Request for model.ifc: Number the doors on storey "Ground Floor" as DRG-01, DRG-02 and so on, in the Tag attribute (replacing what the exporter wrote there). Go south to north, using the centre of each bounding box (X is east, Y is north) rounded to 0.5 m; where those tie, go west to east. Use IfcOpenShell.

First a look at what the model holds.

```python
import ifcopenshell
import ifcopenshell.util.element
import ifcopenshell.util.placement

model = ifcopenshell.open("model.ifc")
print(model.schema)
storey = next(s for s in model.by_type("IfcBuildingStorey") if s.Name == "Ground Floor")
doors = [e for e in ifcopenshell.util.element.get_decomposition(storey) if e.is_a("IfcDoor")]
for e in sorted(doors, key=lambda e: e.id()):
    origin = ifcopenshell.util.placement.get_local_placement(e.ObjectPlacement)[:3, 3]
    print(e.id(), e.Tag, e.Name, origin.round(2) + 0.0, sep=" | ")
```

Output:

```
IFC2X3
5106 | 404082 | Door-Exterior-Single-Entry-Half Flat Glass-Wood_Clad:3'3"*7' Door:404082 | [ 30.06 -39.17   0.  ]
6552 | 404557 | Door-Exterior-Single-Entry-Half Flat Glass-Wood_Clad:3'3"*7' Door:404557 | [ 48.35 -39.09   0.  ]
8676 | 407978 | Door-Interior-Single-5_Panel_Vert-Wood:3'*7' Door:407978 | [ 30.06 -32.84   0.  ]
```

```python
import ifcopenshell
import ifcopenshell.geom
import ifcopenshell.util.element
import ifcopenshell.util.shape

model = ifcopenshell.open("model.ifc")
settings = ifcopenshell.geom.settings()
settings.set("use-world-coords", True)


def centre(element):
    shape = ifcopenshell.geom.create_shape(settings, element)
    return ifcopenshell.util.shape.get_bbox_centroid(shape.geometry)


storey = next(s for s in model.by_type("IfcBuildingStorey") if s.Name == "Ground Floor")
doors = [e for e in ifcopenshell.util.element.get_decomposition(storey) if e.is_a("IfcDoor")]

# Insertion points can sit at a corner or the storey origin, so sort by the geometry (in metres).
centres = {e: centre(e) for e in doors}
doors.sort(key=lambda e: (round(centres[e][1] / 0.5), centres[e][0]))

for i, e in enumerate(doors, start=1):
    number = f"DRG-{i:02d}"
    e.Tag = number
    print(e.id(), number)

model.write("model_updated.ifc")
```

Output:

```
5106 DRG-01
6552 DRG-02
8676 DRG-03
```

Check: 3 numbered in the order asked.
